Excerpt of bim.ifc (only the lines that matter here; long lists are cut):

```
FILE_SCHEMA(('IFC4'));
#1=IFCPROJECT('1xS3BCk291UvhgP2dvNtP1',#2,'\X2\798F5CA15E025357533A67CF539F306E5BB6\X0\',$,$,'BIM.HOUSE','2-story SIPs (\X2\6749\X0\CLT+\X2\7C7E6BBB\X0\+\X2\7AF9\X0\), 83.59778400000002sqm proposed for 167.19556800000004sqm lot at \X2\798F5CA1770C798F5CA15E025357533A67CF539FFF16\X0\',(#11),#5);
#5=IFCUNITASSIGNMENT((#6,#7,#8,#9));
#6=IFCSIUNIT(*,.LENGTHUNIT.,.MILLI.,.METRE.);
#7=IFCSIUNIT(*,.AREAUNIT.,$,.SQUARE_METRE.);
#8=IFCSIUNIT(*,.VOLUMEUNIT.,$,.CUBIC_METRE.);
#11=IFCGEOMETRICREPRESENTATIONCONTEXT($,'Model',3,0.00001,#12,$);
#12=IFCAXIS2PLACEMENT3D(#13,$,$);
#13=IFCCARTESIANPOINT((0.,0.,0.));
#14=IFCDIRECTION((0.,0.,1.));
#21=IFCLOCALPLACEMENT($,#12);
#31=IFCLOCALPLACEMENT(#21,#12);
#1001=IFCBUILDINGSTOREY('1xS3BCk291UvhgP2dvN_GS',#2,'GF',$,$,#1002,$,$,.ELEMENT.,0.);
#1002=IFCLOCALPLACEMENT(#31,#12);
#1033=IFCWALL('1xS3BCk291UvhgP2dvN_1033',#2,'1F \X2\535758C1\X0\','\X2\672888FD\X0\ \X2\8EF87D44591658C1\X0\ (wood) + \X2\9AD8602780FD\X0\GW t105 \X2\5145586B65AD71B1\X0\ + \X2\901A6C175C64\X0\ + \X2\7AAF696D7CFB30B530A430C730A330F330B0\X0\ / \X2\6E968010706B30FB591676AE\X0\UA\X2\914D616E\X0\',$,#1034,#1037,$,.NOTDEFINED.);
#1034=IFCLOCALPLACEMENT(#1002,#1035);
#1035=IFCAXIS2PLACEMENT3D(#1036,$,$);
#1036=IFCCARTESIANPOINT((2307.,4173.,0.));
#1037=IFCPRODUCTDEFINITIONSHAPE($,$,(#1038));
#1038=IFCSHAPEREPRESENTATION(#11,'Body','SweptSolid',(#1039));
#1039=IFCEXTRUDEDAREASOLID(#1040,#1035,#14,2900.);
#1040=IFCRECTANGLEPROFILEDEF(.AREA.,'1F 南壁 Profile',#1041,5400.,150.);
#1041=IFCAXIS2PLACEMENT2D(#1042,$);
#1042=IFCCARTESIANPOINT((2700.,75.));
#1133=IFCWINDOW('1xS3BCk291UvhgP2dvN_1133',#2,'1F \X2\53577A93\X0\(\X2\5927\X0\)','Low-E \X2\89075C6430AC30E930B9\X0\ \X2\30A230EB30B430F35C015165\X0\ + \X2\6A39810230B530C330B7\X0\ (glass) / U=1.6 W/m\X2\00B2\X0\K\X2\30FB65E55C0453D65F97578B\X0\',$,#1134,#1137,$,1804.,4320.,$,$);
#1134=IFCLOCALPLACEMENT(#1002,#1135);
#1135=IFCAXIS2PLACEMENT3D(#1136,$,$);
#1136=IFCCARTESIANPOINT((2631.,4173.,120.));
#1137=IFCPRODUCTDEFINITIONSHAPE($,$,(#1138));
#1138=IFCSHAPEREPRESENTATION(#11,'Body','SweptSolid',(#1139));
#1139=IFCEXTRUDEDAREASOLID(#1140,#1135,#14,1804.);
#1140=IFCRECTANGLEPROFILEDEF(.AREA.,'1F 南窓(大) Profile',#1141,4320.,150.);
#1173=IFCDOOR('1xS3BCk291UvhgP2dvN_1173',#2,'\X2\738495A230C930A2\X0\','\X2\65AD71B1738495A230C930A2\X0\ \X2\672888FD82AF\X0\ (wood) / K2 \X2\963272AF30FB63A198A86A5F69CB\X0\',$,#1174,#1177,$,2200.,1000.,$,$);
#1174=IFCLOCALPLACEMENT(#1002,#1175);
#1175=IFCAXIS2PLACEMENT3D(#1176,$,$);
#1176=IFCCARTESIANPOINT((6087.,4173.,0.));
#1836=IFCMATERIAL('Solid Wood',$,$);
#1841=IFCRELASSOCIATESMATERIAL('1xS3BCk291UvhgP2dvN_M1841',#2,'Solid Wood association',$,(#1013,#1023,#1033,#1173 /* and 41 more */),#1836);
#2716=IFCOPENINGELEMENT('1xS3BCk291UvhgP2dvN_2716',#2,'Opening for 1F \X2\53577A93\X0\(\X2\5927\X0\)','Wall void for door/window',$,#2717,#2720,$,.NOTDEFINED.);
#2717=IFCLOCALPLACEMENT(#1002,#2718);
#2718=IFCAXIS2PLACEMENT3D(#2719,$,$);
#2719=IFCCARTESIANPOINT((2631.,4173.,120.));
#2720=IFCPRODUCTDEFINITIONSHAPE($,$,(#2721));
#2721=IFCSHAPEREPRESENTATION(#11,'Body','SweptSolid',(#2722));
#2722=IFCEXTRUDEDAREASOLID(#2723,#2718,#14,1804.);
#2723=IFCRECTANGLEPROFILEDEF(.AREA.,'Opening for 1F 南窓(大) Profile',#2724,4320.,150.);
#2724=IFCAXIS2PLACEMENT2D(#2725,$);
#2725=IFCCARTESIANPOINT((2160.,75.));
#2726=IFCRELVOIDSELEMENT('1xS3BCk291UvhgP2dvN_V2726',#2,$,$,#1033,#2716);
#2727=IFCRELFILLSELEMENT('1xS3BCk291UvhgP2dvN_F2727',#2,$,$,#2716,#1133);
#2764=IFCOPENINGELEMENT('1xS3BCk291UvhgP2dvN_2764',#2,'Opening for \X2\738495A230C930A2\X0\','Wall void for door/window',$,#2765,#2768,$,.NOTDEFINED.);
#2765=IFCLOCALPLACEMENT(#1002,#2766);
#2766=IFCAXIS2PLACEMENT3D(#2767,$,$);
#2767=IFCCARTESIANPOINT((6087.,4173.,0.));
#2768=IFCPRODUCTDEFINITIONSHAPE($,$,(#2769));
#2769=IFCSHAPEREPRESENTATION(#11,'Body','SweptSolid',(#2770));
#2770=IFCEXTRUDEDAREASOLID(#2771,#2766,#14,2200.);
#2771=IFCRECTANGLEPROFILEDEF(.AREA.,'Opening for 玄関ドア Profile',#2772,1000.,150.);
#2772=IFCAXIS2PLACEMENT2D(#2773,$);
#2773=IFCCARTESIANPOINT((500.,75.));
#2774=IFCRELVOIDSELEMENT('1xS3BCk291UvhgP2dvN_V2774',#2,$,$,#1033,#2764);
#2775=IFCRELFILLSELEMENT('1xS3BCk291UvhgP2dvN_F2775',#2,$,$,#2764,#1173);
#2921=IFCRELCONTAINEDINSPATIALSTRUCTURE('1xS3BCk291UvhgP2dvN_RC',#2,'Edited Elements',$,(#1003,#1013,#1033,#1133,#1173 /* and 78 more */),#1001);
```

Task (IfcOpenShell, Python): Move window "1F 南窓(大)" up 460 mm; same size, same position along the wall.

```python
import numpy as np
import ifcopenshell
import ifcopenshell.api.geometry
import ifcopenshell.util.placement
import ifcopenshell.util.unit

model = ifcopenshell.open("bim.ifc")
unit_scale = ifcopenshell.util.unit.calculate_unit_scale(model)

window = model.by_id(1133)
opening = window.FillsVoids[0].RelatingOpeningElement
dz = 0.46 / unit_scale

shift = np.array([0.0, 0.0, dz])
# The window is not placed relative to its opening, so move both.
for product in (opening, window):
    matrix = ifcopenshell.util.placement.get_local_placement(product.ObjectPlacement)
    matrix[:3, 3] += shift
    ifcopenshell.api.geometry.edit_object_placement(model, product=product, matrix=matrix, is_si=False)

print(f"moved by {dz * unit_scale:+.3f} m")

model.write("bim_edited.ifc")
```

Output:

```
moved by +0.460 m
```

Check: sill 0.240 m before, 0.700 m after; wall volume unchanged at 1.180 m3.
